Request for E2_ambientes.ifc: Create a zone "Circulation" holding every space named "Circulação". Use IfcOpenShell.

First a look at what the model holds.

```python
import ifcopenshell

model = ifcopenshell.open("E2_ambientes.ifc")
print(model.schema)
seen = {}
for space in model.by_type("IfcSpace"):
    seen[space.LongName] = seen.get(space.LongName, 0) + 1
for name, count in sorted(seen.items(), key=str):
    print(count, "x", name)
print("zones:", [z.Name for z in model.by_type("IfcZone")][:20])
```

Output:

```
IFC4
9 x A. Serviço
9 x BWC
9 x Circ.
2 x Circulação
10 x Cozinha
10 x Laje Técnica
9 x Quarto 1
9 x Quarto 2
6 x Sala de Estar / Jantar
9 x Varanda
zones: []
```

```python
import ifcopenshell
import ifcopenshell.api.group
import ifcopenshell.api.root

model = ifcopenshell.open("E2_ambientes.ifc")

names = {"Circulação"}
spaces = [s for s in model.by_type("IfcSpace") if s.LongName in names]

zone = ifcopenshell.api.root.create_entity(model, ifc_class="IfcZone", name="Circulation")
ifcopenshell.api.group.assign_group(model, products=spaces, group=zone)
print(len(spaces), "spaces in", zone.Name)

model.write("E2_ambientes-out.ifc")
```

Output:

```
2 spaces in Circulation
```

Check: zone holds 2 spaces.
